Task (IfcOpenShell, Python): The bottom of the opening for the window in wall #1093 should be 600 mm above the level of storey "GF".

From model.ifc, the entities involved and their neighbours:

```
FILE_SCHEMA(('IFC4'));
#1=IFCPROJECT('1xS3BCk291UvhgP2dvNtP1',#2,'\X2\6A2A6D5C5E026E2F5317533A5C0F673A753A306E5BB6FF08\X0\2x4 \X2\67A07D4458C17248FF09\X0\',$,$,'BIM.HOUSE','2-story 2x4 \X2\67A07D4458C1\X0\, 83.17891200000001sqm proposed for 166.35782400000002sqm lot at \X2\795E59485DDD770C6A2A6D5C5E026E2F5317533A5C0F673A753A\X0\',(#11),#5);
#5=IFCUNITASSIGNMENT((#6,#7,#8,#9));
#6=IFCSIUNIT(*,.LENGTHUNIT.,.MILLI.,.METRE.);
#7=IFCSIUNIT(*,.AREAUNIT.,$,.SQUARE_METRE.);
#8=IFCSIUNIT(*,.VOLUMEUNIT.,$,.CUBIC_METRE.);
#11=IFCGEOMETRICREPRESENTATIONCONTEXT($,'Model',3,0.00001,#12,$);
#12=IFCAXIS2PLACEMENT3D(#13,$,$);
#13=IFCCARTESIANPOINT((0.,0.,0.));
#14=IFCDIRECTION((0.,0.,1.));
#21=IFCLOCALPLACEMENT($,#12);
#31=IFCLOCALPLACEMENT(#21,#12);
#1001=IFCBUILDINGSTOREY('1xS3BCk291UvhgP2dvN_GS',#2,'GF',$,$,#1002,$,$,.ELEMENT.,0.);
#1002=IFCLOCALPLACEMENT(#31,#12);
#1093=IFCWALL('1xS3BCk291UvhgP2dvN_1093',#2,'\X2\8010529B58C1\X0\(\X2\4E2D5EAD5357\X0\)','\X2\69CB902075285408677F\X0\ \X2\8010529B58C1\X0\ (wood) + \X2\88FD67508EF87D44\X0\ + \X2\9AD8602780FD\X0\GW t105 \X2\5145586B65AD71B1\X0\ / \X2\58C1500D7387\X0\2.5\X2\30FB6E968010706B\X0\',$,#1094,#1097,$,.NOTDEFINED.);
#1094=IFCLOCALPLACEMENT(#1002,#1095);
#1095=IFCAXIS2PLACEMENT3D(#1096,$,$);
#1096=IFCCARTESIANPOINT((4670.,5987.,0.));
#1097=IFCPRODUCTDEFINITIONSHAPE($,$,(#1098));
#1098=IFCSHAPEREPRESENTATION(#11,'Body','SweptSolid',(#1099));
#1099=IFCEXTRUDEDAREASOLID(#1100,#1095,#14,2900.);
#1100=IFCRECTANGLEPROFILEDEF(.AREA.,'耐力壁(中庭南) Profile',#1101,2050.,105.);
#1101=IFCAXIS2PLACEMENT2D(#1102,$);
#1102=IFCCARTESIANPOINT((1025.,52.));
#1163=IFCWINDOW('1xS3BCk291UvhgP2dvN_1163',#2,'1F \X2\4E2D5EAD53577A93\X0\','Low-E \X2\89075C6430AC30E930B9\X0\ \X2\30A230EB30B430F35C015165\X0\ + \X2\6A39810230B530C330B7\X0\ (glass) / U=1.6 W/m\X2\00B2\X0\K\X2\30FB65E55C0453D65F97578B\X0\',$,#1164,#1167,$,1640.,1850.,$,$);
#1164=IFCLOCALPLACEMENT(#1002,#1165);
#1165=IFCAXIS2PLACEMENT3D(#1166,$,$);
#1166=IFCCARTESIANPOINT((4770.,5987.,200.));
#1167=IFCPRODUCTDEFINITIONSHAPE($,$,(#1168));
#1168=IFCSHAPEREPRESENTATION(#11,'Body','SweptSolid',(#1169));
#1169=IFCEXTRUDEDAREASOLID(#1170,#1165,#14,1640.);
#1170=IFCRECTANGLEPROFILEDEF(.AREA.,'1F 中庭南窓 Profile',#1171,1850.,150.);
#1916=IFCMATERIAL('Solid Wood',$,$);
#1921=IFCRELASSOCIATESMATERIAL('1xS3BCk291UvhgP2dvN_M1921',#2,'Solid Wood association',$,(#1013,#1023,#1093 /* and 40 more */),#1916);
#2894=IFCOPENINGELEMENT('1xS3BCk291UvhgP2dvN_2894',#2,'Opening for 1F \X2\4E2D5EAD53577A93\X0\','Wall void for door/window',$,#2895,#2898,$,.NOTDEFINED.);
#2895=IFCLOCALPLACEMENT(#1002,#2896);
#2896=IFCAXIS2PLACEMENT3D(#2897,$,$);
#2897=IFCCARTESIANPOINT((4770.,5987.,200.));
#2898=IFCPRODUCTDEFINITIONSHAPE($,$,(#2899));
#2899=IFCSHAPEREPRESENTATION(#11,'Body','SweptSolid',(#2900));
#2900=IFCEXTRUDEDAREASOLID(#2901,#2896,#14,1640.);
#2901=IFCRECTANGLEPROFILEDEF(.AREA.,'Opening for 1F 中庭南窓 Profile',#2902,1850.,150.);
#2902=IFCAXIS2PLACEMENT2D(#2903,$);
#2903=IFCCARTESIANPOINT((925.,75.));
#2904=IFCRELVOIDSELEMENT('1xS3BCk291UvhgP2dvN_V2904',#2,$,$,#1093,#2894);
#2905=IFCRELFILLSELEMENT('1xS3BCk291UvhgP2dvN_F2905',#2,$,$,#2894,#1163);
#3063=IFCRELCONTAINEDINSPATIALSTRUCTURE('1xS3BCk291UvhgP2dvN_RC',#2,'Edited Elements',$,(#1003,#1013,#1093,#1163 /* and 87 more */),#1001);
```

```python
import numpy as np
import ifcopenshell
import ifcopenshell.api.geometry
import ifcopenshell.geom
import ifcopenshell.util.element
import ifcopenshell.util.placement
import ifcopenshell.util.shape
import ifcopenshell.util.unit

model = ifcopenshell.open("model.ifc")
unit_scale = ifcopenshell.util.unit.calculate_unit_scale(model)

window = model.by_guid("1xS3BCk291UvhgP2dvN_1163")
opening = window.FillsVoids[0].RelatingOpeningElement
storey = ifcopenshell.util.element.get_container(window, ifc_class="IfcBuildingStorey")
level = ifcopenshell.util.placement.get_local_placement(storey.ObjectPlacement)[2, 3]

# The opening's origin need not be at the sill, so measure its lowest point.
shape = ifcopenshell.geom.create_shape(ifcopenshell.geom.settings(), opening)
bottom = ifcopenshell.util.shape.get_shape_bottom_elevation(shape, shape.geometry) / unit_scale
dz = level + 600.0 - bottom

shift = np.array([0.0, 0.0, dz])
# The window is not placed relative to its opening, so move both.
for product in (opening, window):
    matrix = ifcopenshell.util.placement.get_local_placement(product.ObjectPlacement)
    matrix[:3, 3] += shift
    ifcopenshell.api.geometry.edit_object_placement(model, product=product, matrix=matrix, is_si=False)

print(f"moved by {dz * unit_scale:+.3f} m")

model.write("model-out.ifc")
```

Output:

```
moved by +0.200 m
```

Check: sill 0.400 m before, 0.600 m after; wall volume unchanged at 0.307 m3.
